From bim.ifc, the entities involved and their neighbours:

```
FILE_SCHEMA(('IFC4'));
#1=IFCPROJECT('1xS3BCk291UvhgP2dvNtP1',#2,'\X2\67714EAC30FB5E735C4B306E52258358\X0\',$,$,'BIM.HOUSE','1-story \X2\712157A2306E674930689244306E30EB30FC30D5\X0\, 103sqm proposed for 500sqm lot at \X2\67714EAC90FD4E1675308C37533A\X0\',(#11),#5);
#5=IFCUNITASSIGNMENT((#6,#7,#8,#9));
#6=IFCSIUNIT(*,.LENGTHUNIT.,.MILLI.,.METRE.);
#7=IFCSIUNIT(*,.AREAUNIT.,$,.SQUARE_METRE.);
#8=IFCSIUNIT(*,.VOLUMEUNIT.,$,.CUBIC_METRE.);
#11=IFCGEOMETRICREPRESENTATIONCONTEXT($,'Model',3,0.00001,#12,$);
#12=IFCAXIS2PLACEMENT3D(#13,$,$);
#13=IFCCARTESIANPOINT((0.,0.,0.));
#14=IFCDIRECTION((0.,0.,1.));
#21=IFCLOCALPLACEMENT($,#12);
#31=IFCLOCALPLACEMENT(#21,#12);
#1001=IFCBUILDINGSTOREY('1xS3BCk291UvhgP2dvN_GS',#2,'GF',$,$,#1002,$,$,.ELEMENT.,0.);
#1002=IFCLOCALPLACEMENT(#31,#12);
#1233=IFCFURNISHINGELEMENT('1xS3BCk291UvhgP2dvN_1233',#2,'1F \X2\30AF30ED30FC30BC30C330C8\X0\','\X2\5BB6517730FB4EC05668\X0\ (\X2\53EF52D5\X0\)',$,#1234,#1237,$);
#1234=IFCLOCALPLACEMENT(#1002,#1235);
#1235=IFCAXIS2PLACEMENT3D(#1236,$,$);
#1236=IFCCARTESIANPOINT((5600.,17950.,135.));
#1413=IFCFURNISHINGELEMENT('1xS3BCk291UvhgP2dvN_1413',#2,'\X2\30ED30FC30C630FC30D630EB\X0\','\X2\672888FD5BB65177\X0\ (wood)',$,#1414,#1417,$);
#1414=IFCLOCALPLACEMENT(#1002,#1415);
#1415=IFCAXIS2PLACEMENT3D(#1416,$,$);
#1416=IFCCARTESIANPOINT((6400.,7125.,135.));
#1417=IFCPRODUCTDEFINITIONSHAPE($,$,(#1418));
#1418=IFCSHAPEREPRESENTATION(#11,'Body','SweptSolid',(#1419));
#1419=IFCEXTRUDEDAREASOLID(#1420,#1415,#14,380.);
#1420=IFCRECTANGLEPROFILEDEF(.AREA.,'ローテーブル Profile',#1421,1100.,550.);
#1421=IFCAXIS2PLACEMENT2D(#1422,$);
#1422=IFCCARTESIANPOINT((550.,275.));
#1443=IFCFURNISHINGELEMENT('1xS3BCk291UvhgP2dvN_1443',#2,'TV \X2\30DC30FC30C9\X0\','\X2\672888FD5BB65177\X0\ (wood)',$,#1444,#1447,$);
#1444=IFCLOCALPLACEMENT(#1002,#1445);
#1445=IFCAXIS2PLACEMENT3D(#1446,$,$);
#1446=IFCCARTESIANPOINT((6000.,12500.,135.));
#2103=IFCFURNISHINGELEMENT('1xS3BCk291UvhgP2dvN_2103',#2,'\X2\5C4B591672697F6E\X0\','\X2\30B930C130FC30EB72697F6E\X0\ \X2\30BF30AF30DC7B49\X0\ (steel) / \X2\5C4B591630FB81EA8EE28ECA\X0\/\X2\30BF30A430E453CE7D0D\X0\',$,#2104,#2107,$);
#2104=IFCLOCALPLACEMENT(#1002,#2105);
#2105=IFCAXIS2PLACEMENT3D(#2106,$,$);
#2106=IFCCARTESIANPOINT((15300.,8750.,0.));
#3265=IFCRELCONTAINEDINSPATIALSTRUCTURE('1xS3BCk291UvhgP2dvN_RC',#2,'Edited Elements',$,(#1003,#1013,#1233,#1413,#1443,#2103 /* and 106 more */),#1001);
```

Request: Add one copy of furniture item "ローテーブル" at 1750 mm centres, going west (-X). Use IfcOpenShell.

```python
import numpy as np
import ifcopenshell
import ifcopenshell.api.geometry
import ifcopenshell.api.root
import ifcopenshell.util.element
import ifcopenshell.util.placement
import ifcopenshell.util.unit

model = ifcopenshell.open("bim.ifc")
unit_scale = ifcopenshell.util.unit.calculate_unit_scale(model)


def reuse_history(source, copy):
    """copy_class also copies each property set's owner history, people and application; keep the originals."""
    for rel in copy.IsDefinedBy:
        if rel.is_a("IfcRelDefinesByProperties") and (history := rel.RelatingPropertyDefinition.OwnerHistory):
            rel.RelatingPropertyDefinition.OwnerHistory = source.OwnerHistory
            ifcopenshell.util.element.remove_deep2(model, history)


source = model.by_guid("1xS3BCk291UvhgP2dvN_1413")
base = ifcopenshell.util.placement.get_local_placement(source.ObjectPlacement)
step = np.array([-1.0, 0.0, 0.0]) * 1.75 / unit_scale

for i in range(1, 2):
    copy = ifcopenshell.api.root.copy_class(model, product=source)
    copy.Representation = ifcopenshell.util.element.copy_deep(
        model, source.Representation, exclude=["IfcGeometricRepresentationContext", "IfcRepresentationMap"]
    )
    reuse_history(source, copy)
    matrix = base.copy()
    matrix[:3, 3] += i * step
    print("added at", matrix[:3, 3].round(3) + 0.0)
    ifcopenshell.api.geometry.edit_object_placement(model, product=copy, matrix=matrix, is_si=False)

model.write("bim_v2.ifc")
```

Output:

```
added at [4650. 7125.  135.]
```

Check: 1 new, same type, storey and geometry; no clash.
